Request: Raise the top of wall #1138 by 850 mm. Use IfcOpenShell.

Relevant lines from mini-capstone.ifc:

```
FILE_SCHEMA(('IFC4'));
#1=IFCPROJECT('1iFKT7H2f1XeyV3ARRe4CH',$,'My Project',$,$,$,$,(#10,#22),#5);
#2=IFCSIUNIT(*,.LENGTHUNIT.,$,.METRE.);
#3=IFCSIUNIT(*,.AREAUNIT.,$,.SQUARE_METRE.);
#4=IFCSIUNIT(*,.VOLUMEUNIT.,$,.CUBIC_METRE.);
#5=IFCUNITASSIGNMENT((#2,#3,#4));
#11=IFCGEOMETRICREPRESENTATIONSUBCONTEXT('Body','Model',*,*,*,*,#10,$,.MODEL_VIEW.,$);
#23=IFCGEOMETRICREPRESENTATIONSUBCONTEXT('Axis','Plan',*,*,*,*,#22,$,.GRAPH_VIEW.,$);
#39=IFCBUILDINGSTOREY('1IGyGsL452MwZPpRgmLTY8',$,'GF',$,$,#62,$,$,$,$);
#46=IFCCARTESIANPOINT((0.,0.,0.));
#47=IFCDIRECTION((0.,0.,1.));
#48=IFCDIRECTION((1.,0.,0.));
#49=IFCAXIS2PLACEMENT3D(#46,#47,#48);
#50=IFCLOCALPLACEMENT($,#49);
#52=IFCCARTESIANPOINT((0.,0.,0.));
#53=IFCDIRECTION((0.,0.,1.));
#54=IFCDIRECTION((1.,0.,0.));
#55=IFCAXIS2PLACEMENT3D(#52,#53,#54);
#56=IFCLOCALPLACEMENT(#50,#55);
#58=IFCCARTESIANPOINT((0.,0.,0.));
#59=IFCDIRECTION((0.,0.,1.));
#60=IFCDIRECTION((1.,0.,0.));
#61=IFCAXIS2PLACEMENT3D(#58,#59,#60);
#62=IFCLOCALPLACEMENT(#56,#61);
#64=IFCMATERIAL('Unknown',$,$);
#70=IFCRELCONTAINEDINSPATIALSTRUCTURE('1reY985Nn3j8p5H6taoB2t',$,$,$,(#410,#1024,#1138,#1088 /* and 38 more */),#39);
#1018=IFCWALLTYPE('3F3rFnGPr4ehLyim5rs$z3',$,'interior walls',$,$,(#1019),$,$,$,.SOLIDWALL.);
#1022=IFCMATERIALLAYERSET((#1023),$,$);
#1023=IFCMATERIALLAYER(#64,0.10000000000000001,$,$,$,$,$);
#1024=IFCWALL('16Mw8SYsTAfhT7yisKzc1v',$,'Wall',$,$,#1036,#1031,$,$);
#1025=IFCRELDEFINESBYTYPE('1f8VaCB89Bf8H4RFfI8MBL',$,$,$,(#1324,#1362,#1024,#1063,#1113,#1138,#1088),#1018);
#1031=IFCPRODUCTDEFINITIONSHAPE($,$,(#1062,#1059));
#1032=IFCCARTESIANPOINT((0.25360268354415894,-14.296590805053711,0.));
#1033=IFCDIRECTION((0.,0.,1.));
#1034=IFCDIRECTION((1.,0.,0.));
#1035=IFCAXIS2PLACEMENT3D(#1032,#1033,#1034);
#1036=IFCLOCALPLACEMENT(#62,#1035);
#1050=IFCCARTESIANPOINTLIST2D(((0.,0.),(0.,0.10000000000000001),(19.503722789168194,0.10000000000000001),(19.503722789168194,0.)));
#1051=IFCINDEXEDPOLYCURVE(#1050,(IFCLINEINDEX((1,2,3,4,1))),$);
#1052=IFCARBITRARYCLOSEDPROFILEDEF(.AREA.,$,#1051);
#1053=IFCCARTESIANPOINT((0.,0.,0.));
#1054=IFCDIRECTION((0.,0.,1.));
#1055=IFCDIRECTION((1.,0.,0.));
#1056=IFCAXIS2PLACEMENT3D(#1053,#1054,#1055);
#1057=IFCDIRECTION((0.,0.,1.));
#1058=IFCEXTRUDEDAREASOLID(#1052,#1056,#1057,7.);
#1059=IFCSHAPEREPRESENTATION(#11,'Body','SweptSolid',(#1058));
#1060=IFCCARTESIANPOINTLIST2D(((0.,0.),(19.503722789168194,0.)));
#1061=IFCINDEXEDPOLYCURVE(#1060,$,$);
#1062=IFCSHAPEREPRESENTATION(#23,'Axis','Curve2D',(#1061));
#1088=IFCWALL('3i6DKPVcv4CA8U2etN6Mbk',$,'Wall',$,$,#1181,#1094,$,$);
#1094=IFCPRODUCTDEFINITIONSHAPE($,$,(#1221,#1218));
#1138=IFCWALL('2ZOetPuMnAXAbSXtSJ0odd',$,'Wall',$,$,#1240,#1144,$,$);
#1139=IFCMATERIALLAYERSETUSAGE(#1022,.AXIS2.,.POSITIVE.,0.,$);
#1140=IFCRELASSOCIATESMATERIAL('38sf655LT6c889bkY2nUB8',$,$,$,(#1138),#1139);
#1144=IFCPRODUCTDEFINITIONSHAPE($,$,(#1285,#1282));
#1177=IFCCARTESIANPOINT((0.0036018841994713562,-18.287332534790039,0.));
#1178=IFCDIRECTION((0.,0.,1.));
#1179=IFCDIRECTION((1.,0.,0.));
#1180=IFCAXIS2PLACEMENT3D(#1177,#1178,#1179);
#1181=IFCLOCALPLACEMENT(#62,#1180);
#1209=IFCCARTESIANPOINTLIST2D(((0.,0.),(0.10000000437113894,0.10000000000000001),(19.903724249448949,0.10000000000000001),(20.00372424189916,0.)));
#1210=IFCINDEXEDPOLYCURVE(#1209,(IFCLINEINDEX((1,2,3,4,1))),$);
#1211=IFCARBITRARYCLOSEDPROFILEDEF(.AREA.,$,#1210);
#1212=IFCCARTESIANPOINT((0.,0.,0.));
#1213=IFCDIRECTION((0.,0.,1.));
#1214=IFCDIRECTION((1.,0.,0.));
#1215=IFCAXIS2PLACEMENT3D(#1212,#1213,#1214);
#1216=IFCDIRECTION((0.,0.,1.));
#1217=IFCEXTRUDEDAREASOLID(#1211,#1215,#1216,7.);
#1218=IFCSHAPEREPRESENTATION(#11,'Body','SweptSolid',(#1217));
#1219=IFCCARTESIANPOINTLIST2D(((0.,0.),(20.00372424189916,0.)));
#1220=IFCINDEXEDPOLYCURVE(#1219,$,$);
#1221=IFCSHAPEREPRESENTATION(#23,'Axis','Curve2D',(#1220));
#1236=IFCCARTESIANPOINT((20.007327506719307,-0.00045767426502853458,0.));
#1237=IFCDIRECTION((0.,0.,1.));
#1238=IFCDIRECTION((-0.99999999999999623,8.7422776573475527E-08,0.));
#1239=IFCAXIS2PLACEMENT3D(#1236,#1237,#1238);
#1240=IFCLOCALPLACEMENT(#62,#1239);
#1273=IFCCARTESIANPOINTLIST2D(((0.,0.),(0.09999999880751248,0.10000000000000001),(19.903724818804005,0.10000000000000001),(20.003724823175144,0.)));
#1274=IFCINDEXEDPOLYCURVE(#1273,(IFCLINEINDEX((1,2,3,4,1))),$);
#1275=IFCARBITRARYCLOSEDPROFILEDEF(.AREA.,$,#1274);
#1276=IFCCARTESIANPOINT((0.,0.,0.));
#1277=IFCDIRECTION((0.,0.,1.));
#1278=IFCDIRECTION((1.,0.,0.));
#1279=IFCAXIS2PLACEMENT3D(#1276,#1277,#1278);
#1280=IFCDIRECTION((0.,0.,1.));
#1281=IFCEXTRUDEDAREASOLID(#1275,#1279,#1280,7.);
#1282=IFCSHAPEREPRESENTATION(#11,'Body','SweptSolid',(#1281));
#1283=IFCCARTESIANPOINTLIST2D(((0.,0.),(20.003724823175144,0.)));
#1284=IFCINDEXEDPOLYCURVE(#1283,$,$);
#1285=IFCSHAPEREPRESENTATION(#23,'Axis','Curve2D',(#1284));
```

```python
import ifcopenshell
import ifcopenshell.geom
import ifcopenshell.util.representation
import ifcopenshell.util.shape
import ifcopenshell.util.unit

model = ifcopenshell.open("mini-capstone.ifc")
unit_scale = ifcopenshell.util.unit.calculate_unit_scale(model)
settings = ifcopenshell.geom.settings()


def volume(element):
    """Net volume in cubic metres, openings subtracted."""
    shape = ifcopenshell.geom.create_shape(settings, element)
    return ifcopenshell.util.shape.get_volume(shape.geometry)


wall = model.by_guid("2ZOetPuMnAXAbSXtSJ0odd")
before = volume(wall)

body = ifcopenshell.util.representation.get_representation(wall, "Model", "Body")
solid = body.Items[0]
old_height = solid.Depth
solid.Depth += 0.85 / unit_scale
after = volume(wall)

print(f"height {old_height:g} -> {solid.Depth:g}, volume {before:.3f} -> {after:.3f} m3")

model.write("mini-capstone_updated.ifc")
```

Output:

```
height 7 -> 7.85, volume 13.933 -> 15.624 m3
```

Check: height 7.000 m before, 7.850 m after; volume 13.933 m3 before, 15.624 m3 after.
